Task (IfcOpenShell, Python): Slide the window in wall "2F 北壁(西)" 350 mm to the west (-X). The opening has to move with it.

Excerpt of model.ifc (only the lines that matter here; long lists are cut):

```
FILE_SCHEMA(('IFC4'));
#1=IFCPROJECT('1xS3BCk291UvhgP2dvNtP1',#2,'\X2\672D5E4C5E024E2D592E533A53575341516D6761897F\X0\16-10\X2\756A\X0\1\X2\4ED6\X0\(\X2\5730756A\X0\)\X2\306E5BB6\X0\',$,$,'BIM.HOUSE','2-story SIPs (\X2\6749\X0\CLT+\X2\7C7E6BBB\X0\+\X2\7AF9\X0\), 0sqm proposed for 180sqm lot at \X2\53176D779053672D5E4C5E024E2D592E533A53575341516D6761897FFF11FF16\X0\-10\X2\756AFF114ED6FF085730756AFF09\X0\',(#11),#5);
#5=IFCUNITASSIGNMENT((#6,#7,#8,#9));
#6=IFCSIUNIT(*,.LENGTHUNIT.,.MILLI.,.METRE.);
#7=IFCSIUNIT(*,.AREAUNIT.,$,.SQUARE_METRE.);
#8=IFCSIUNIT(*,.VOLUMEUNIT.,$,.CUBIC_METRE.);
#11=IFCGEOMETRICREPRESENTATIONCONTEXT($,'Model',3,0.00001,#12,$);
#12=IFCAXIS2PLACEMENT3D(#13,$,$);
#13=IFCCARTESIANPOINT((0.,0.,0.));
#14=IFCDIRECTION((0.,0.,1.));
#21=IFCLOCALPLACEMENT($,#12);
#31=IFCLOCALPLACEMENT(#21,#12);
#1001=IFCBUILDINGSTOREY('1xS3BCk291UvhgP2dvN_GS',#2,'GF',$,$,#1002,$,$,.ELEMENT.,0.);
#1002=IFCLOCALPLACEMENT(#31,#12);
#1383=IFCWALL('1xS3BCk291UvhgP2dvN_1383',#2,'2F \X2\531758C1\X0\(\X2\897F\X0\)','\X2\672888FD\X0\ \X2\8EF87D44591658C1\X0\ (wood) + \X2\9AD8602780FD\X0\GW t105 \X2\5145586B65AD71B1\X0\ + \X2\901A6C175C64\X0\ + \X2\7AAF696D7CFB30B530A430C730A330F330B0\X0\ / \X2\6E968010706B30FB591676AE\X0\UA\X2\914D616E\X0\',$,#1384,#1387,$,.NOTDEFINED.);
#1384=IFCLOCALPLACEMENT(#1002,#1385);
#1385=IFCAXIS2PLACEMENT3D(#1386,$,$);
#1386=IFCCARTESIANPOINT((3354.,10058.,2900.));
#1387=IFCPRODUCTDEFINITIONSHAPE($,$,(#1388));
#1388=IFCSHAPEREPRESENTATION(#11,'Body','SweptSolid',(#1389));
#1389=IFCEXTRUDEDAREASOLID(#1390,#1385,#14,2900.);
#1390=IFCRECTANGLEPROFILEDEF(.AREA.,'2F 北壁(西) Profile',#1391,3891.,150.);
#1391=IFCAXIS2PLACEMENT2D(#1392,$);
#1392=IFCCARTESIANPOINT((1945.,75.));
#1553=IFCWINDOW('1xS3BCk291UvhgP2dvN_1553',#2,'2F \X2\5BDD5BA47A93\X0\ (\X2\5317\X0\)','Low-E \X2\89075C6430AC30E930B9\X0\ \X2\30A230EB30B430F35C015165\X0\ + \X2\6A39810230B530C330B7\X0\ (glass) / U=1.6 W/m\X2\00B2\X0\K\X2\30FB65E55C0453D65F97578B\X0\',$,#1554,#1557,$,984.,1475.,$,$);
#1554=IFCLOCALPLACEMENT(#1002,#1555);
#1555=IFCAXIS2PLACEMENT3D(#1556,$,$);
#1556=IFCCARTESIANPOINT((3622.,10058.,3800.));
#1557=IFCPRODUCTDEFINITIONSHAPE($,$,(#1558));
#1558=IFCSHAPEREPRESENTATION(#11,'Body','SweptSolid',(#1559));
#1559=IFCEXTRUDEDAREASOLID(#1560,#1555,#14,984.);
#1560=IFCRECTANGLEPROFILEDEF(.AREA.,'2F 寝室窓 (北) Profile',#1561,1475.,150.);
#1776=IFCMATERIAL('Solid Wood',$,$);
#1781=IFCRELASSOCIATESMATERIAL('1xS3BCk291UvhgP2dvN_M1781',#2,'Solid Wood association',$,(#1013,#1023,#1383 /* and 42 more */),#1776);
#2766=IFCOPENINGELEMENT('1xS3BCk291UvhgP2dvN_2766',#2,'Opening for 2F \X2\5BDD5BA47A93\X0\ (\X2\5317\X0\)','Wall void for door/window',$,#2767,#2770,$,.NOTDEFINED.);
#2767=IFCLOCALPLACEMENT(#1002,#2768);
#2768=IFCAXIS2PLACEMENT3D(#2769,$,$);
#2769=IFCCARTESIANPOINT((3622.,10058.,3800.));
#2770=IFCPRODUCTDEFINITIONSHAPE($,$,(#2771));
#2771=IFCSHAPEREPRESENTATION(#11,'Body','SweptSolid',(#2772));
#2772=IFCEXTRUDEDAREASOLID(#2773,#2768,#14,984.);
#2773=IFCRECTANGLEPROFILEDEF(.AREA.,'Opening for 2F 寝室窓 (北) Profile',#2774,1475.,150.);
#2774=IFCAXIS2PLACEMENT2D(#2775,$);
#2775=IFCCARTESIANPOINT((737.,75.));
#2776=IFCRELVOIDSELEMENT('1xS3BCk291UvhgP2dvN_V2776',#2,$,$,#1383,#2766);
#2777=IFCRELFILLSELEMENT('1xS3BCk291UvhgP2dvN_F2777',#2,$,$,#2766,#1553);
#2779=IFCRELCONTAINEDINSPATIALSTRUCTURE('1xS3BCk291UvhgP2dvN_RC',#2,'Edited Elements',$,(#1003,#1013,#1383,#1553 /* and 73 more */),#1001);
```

```python
import ifcopenshell
import ifcopenshell.api.geometry
import ifcopenshell.util.placement
import ifcopenshell.util.unit

model = ifcopenshell.open("model.ifc")
unit_scale = ifcopenshell.util.unit.calculate_unit_scale(model)

window = model.by_guid("1xS3BCk291UvhgP2dvN_1553")
opening = window.FillsVoids[0].RelatingOpeningElement
wall = opening.VoidsElements[0].RelatingBuildingElement

wall_matrix = ifcopenshell.util.placement.get_local_placement(wall.ObjectPlacement)
shift = wall_matrix[:3, 0] * -0.35 / unit_scale
before = ifcopenshell.util.placement.get_local_placement(window.ObjectPlacement)[:3, 3].copy()

# The window is not placed relative to its opening, so move both.
for product in (opening, window):
    matrix = ifcopenshell.util.placement.get_local_placement(product.ObjectPlacement)
    matrix[:3, 3] += shift
    ifcopenshell.api.geometry.edit_object_placement(model, product=product, matrix=matrix, is_si=False)

after = ifcopenshell.util.placement.get_local_placement(window.ObjectPlacement)[:3, 3]
print("window moved by", (after - before).round(3) + 0.0)

model.write("model_updated.ifc")
```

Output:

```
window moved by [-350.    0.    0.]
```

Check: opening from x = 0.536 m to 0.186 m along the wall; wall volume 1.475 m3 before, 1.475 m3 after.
